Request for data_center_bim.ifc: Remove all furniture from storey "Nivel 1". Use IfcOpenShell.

First a look at what the model holds.

```python
import ifcopenshell
import ifcopenshell.util.element

model = ifcopenshell.open("data_center_bim.ifc")
print(model.schema)
storey = next(s for s in model.by_type("IfcBuildingStorey") if s.Name == "Nivel 1")
furniture = [e for e in ifcopenshell.util.element.get_decomposition(storey) if e.is_a("IfcFurnishingElement")]
seen = {}
for e in furniture:
    element_type = ifcopenshell.util.element.get_type(e)
    name = element_type.Name if element_type not in (None, e) else None
    seen[name] = seen.get(name, 0) + 1
for name, count in sorted(seen.items(), key=str):
    print(count, "x", name)
```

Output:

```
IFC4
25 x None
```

```python
import ifcopenshell
import ifcopenshell.api.root
import ifcopenshell.util.element

model = ifcopenshell.open("data_center_bim.ifc")

storey = next(s for s in model.by_type("IfcBuildingStorey") if s.Name == "Nivel 1")
furniture = [e for e in ifcopenshell.util.element.get_decomposition(storey) if e.is_a("IfcFurnishingElement")]

for e in furniture:
    ifcopenshell.api.root.remove_product(model, product=e)
print(len(furniture), "removed")

model.write("data_center_bim-out.ifc")
```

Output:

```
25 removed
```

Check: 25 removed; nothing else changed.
